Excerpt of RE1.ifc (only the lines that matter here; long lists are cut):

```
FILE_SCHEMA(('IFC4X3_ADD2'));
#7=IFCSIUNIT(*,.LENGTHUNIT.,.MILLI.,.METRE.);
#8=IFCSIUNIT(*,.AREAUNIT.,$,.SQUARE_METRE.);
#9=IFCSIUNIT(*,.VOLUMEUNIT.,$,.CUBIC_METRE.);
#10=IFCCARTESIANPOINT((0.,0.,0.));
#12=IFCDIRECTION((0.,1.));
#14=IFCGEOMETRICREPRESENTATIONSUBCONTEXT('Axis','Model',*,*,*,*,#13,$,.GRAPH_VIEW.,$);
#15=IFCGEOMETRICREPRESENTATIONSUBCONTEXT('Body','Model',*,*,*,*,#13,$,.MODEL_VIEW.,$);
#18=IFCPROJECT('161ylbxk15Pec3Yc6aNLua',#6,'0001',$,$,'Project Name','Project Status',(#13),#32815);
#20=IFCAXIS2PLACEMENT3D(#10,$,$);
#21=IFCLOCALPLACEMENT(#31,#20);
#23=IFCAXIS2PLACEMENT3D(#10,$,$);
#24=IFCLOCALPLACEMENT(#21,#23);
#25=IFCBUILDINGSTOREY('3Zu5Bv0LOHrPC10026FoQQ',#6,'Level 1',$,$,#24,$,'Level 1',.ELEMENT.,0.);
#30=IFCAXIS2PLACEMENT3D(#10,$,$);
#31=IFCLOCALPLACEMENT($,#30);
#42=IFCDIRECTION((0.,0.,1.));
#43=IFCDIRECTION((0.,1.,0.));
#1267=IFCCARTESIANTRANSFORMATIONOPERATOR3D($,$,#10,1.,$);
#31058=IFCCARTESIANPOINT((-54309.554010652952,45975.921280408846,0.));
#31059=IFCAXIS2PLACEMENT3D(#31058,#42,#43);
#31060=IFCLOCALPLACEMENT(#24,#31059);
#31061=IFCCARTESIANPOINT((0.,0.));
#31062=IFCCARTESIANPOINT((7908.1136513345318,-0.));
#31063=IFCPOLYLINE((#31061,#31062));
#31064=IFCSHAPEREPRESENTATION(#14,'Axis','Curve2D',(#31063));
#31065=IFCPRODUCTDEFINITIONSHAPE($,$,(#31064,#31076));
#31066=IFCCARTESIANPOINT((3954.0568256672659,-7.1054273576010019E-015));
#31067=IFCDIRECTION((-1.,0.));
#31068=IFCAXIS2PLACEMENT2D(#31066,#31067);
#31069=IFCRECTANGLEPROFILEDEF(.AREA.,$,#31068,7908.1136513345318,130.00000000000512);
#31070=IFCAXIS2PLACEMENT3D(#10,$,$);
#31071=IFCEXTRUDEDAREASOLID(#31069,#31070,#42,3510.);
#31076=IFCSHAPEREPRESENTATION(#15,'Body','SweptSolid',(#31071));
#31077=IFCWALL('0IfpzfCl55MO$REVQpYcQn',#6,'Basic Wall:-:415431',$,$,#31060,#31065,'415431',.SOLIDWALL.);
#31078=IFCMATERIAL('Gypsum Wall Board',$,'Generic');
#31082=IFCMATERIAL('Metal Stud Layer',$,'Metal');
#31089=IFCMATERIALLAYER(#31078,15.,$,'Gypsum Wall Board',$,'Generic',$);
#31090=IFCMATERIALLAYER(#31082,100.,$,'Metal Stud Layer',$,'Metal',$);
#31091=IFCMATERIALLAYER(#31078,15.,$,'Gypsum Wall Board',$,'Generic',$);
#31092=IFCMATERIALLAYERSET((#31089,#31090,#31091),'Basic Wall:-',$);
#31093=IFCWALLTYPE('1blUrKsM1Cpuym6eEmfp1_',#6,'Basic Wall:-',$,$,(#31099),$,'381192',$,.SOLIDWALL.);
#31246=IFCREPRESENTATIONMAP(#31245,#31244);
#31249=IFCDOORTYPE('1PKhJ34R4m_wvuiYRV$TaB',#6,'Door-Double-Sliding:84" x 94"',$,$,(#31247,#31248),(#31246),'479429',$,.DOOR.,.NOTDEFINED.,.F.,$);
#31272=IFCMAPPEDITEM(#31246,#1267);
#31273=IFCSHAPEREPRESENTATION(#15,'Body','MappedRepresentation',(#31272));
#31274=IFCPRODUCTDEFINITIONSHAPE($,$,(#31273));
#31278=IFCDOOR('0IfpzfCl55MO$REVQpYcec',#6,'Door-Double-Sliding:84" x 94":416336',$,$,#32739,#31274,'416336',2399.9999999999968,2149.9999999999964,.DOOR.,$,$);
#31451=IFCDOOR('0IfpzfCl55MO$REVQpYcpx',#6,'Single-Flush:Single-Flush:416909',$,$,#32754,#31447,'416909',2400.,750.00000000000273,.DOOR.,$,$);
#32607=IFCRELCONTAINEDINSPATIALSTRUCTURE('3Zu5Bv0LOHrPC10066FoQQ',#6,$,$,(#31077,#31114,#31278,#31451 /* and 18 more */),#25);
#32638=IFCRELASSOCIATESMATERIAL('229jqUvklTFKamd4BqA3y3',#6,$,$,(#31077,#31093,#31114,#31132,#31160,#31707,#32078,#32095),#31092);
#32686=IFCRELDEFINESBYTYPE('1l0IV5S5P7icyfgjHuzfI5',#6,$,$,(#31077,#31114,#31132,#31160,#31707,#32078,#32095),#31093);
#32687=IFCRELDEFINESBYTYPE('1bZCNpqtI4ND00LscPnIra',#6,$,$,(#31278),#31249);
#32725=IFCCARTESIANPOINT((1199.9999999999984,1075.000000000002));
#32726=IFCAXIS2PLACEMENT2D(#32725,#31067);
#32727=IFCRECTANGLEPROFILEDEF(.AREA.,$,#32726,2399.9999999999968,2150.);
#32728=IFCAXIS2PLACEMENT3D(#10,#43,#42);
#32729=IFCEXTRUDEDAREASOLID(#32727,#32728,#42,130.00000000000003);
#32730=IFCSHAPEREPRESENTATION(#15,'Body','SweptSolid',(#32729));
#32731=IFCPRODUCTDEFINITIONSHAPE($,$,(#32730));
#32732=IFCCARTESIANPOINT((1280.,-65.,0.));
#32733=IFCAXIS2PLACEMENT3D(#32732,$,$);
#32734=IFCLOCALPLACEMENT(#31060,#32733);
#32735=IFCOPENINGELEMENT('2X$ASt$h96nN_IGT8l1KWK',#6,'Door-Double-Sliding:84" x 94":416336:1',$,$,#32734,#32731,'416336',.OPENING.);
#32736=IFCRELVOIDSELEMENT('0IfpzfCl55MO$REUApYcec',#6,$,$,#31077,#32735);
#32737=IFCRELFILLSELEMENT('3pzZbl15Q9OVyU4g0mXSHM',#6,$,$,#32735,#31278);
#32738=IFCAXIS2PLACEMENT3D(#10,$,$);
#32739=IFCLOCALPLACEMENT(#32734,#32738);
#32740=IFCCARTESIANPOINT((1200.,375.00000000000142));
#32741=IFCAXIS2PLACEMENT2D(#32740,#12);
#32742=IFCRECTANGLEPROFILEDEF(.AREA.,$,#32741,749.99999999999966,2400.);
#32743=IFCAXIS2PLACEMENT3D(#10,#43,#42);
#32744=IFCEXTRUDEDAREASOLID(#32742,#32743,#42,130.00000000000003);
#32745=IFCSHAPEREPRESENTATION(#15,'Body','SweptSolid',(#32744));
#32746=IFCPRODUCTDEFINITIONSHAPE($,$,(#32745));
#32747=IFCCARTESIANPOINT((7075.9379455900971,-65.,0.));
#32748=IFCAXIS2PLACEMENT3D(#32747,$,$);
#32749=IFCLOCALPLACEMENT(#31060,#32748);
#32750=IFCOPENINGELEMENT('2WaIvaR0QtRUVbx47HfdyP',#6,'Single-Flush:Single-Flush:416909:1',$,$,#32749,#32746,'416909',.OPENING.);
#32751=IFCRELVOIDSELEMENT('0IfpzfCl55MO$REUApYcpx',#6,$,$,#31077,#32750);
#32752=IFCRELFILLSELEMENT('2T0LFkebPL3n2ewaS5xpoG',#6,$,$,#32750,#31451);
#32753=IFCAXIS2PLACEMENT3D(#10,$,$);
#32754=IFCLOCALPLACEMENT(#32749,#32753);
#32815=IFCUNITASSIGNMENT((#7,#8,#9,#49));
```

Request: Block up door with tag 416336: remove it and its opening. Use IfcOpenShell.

```python
import ifcopenshell
import ifcopenshell.api.feature
import ifcopenshell.api.root
import ifcopenshell.geom
import ifcopenshell.util.shape

model = ifcopenshell.open("RE1.ifc")
settings = ifcopenshell.geom.settings()


def volume(element):
    """Net volume in cubic metres, openings subtracted."""
    shape = ifcopenshell.geom.create_shape(settings, element)
    return ifcopenshell.util.shape.get_volume(shape.geometry)


door = model.by_guid("0IfpzfCl55MO$REVQpYcec")
opening = door.FillsVoids[0].RelatingOpeningElement
wall = opening.VoidsElements[0].RelatingBuildingElement
before = volume(wall)

ifcopenshell.api.root.remove_product(model, product=door)
ifcopenshell.api.feature.remove_feature(model, feature=opening)

after = volume(wall)

print(f"wall volume {before:.3f} -> {after:.3f} m3")

model.write("RE1-out.ifc")
```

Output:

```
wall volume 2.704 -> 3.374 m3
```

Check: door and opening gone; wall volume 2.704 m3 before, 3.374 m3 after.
